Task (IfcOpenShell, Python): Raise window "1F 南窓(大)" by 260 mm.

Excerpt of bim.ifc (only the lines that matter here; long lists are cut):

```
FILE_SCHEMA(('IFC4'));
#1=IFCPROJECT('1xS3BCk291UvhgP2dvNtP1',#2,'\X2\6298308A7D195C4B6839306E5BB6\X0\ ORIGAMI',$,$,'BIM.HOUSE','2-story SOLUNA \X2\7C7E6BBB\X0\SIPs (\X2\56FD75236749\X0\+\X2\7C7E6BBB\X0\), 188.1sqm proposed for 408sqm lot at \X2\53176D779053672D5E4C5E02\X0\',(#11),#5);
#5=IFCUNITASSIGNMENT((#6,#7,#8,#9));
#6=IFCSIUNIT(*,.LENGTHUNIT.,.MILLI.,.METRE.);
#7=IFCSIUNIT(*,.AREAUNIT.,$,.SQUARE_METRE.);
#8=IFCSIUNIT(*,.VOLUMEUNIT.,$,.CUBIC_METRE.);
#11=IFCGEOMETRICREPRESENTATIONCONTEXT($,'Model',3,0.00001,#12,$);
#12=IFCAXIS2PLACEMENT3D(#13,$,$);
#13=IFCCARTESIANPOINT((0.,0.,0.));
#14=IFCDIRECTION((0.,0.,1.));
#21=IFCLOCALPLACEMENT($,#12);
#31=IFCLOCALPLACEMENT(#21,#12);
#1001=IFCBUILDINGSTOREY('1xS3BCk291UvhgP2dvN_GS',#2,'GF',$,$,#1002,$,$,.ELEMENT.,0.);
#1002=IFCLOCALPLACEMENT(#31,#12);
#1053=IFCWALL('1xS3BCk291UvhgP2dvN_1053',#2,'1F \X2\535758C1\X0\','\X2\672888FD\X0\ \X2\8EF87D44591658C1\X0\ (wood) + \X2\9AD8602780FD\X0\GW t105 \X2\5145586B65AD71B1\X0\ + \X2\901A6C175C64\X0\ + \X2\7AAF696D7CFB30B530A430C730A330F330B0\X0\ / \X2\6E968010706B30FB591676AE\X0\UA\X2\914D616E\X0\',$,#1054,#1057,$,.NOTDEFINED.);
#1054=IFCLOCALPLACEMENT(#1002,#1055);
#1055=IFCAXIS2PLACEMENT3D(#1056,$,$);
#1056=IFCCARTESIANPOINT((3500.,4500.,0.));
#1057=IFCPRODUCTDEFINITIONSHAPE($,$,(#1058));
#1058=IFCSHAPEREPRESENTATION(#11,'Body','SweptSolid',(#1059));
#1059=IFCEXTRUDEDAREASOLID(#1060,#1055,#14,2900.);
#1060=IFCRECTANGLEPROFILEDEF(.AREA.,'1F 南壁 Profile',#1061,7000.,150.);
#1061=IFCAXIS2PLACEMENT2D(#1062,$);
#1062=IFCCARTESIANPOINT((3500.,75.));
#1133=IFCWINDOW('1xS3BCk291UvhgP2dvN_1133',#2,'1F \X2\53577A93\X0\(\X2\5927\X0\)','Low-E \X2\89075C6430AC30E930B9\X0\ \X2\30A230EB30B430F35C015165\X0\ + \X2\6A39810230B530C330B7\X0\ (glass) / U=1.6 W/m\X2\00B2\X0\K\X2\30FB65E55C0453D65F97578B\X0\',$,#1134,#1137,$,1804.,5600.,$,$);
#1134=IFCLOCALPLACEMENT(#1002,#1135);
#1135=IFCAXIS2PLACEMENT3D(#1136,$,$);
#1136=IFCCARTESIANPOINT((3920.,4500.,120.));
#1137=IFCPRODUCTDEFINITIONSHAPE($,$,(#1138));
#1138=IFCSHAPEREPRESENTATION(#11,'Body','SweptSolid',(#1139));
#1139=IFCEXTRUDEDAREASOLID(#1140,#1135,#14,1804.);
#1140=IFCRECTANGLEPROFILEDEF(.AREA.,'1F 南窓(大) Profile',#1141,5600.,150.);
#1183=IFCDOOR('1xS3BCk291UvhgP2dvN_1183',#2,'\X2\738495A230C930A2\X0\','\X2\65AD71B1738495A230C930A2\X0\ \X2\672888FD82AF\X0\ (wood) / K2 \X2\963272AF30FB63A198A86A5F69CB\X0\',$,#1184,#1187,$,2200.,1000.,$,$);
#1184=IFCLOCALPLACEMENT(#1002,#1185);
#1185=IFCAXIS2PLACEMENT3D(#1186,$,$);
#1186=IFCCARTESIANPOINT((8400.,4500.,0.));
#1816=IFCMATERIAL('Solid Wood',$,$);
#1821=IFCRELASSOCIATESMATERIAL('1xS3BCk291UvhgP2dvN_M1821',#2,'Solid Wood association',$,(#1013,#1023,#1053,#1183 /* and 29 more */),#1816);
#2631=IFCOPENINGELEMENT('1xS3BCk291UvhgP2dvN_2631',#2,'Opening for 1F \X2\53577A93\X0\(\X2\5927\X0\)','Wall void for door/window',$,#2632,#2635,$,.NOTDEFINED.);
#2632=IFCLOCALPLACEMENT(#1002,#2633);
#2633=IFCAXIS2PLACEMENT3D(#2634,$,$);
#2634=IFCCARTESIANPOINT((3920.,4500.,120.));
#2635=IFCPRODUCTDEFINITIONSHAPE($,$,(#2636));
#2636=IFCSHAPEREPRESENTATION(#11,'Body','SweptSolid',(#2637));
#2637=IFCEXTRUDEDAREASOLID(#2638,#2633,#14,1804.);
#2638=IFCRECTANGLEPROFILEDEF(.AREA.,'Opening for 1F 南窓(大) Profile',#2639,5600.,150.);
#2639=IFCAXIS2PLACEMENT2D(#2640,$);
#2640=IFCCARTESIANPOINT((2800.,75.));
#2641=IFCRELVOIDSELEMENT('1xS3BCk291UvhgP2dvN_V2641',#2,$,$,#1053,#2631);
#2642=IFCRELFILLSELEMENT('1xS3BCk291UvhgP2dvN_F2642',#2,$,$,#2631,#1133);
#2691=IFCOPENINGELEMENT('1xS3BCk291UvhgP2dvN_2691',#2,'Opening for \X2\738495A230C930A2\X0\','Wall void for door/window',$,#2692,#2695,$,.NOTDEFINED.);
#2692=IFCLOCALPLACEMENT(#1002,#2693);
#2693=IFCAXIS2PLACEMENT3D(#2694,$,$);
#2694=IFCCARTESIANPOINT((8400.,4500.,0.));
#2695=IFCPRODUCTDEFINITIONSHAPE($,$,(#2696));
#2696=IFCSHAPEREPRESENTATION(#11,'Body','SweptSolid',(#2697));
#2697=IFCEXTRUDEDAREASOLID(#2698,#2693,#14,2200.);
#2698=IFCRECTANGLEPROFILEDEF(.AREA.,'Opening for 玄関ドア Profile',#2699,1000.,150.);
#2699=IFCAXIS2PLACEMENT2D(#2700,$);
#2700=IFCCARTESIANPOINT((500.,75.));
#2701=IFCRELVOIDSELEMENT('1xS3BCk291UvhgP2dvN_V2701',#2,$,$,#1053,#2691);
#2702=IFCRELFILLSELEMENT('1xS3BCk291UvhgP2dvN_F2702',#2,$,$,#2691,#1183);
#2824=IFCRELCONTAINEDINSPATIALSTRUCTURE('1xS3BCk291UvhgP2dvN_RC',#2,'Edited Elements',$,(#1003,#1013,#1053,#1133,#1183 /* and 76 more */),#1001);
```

```python
import numpy as np
import ifcopenshell
import ifcopenshell.api.geometry
import ifcopenshell.util.placement
import ifcopenshell.util.unit

model = ifcopenshell.open("bim.ifc")
unit_scale = ifcopenshell.util.unit.calculate_unit_scale(model)

window = model.by_guid("1xS3BCk291UvhgP2dvN_1133")
opening = window.FillsVoids[0].RelatingOpeningElement
dz = 260.0

shift = np.array([0.0, 0.0, dz])
# The window is not placed relative to its opening, so move both.
for product in (opening, window):
    matrix = ifcopenshell.util.placement.get_local_placement(product.ObjectPlacement)
    matrix[:3, 3] += shift
    ifcopenshell.api.geometry.edit_object_placement(model, product=product, matrix=matrix, is_si=False)

print(f"moved by {dz * unit_scale:+.3f} m")

model.write("bim_edited.ifc")
```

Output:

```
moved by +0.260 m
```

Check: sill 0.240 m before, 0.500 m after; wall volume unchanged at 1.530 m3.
